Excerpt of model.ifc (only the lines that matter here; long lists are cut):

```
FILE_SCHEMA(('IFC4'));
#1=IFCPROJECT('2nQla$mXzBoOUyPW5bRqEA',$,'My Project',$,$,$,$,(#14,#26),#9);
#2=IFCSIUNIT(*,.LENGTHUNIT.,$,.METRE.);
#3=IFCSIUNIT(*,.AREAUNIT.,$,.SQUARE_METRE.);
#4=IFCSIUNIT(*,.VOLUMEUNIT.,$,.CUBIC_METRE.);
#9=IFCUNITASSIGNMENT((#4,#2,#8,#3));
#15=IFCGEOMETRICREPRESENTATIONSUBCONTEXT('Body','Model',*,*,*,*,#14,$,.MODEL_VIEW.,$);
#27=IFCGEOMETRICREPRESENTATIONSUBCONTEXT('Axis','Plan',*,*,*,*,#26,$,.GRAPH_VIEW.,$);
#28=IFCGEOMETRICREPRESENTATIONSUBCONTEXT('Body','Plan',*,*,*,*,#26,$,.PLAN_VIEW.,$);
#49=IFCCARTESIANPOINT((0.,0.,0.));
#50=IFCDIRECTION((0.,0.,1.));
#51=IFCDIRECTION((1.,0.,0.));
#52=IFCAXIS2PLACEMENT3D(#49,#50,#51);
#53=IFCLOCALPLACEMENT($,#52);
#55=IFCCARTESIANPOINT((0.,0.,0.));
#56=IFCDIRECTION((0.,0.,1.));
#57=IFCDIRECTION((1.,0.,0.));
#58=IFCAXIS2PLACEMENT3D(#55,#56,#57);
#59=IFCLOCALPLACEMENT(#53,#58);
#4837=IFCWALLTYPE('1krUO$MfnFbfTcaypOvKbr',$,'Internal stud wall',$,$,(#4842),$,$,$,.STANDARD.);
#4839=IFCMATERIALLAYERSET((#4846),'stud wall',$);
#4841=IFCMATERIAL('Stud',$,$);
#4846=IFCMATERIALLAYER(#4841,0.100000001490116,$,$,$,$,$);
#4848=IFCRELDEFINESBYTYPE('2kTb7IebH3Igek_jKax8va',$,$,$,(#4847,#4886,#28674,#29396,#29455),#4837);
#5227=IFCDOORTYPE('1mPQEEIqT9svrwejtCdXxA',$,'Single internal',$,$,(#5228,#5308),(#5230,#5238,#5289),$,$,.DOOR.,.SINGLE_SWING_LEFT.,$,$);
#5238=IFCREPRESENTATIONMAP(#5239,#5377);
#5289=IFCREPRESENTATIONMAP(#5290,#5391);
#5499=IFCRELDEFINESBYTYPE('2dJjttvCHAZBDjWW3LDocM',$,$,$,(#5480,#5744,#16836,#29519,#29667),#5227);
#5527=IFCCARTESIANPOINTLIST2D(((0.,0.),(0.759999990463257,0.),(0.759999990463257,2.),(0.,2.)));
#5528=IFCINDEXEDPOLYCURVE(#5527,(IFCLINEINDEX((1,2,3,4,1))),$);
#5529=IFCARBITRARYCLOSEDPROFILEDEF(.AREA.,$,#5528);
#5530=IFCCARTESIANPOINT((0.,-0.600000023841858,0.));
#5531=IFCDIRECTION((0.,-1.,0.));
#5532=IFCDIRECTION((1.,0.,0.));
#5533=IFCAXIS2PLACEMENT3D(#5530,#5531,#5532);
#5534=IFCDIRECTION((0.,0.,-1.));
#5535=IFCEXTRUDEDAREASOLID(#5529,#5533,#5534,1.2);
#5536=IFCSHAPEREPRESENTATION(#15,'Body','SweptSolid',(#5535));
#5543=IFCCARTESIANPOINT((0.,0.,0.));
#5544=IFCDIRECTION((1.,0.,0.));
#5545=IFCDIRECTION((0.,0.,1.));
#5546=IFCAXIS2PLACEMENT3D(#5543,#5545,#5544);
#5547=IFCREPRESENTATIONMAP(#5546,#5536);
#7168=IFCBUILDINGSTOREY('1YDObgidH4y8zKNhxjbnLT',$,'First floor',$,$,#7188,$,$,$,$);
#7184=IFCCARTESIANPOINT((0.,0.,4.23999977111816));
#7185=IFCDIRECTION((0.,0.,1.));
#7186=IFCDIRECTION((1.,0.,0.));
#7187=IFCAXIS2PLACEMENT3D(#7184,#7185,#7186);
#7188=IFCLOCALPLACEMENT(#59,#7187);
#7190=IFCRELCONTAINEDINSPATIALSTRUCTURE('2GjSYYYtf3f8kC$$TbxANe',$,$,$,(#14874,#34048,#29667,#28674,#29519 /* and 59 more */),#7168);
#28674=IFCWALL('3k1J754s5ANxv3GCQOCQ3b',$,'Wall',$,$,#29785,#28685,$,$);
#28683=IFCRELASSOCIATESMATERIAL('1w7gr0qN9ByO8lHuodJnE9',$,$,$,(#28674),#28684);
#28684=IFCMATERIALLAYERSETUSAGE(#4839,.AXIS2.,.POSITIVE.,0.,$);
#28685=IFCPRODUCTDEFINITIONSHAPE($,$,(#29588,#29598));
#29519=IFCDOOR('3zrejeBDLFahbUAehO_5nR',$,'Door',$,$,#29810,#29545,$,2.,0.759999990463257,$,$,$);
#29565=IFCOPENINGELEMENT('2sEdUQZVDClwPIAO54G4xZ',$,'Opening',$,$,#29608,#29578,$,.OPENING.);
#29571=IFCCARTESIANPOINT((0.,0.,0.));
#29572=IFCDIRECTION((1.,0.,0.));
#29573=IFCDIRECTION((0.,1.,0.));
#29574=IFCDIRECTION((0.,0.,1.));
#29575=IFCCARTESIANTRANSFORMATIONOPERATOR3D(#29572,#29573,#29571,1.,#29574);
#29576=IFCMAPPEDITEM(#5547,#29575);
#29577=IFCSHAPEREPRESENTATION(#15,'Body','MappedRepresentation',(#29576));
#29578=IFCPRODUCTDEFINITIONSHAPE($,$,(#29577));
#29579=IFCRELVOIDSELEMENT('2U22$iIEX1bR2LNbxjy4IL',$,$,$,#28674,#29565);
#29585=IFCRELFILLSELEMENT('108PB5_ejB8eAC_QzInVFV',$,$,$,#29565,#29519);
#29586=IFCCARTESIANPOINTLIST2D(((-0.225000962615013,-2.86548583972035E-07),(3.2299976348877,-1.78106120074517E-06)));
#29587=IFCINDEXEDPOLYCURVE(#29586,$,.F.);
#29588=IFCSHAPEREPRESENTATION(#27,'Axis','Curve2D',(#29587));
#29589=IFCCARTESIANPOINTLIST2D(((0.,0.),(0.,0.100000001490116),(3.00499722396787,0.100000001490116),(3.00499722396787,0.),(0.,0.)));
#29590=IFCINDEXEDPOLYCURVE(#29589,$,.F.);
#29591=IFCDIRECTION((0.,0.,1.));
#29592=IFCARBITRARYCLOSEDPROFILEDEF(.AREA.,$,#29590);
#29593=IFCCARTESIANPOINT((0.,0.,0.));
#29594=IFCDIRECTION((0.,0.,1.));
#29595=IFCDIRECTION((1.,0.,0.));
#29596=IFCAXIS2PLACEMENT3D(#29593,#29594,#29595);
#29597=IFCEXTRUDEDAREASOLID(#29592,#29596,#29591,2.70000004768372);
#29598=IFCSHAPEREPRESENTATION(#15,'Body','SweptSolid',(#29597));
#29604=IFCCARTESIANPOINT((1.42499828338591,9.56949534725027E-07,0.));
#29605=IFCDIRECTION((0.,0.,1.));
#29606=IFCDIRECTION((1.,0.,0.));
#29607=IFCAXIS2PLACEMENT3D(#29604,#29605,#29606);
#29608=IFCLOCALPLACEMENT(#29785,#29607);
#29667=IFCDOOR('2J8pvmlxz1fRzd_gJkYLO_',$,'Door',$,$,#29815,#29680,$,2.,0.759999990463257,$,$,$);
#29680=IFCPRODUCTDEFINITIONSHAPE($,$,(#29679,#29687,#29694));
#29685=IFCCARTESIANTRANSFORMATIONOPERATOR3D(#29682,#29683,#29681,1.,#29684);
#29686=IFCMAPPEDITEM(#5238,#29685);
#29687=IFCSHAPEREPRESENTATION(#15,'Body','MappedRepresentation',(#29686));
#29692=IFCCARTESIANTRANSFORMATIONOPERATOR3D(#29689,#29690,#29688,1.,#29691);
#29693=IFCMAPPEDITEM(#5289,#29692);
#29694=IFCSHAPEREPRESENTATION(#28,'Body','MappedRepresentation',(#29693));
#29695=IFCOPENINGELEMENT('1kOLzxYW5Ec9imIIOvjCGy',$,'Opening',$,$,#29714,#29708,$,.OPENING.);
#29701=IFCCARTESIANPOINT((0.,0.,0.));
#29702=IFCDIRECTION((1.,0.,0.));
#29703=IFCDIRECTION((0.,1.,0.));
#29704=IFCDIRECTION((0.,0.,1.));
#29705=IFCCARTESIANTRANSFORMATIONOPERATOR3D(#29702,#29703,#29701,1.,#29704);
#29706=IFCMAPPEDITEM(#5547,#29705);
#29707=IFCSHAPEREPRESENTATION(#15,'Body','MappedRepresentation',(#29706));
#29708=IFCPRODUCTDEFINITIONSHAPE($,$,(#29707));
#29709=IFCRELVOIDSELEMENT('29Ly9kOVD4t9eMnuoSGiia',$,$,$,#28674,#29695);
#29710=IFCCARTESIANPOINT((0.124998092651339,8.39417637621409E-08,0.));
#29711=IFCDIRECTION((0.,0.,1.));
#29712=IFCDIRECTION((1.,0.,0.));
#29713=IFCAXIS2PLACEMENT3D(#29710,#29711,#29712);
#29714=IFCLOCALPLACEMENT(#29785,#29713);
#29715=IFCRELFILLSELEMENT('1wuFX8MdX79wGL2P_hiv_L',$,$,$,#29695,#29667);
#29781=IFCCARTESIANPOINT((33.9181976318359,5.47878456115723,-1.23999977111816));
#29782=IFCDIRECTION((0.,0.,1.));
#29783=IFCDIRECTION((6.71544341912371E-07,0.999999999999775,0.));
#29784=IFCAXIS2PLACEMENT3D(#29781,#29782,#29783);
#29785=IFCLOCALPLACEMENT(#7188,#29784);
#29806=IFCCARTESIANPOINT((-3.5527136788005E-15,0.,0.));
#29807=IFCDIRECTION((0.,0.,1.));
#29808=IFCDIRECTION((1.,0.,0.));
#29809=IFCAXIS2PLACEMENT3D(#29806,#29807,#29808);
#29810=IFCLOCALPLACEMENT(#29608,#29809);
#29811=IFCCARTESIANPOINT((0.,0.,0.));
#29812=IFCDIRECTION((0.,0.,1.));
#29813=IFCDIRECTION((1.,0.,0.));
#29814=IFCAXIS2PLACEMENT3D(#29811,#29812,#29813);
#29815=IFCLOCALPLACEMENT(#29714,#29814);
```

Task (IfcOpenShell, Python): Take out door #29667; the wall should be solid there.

```python
import ifcopenshell
import ifcopenshell.api.feature
import ifcopenshell.api.root
import ifcopenshell.geom
import ifcopenshell.util.shape

model = ifcopenshell.open("model.ifc")
settings = ifcopenshell.geom.settings()


def volume(element):
    """Net volume in cubic metres, openings subtracted."""
    shape = ifcopenshell.geom.create_shape(settings, element)
    return ifcopenshell.util.shape.get_volume(shape.geometry)


door = model.by_id(29667)
opening = door.FillsVoids[0].RelatingOpeningElement
wall = opening.VoidsElements[0].RelatingBuildingElement
before = volume(wall)

ifcopenshell.api.root.remove_product(model, product=door)
ifcopenshell.api.feature.remove_feature(model, feature=opening)

after = volume(wall)

print(f"wall volume {before:.3f} -> {after:.3f} m3")

model.write("model_v2.ifc")
```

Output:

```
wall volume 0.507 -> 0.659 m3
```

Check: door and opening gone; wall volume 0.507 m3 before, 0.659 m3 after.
